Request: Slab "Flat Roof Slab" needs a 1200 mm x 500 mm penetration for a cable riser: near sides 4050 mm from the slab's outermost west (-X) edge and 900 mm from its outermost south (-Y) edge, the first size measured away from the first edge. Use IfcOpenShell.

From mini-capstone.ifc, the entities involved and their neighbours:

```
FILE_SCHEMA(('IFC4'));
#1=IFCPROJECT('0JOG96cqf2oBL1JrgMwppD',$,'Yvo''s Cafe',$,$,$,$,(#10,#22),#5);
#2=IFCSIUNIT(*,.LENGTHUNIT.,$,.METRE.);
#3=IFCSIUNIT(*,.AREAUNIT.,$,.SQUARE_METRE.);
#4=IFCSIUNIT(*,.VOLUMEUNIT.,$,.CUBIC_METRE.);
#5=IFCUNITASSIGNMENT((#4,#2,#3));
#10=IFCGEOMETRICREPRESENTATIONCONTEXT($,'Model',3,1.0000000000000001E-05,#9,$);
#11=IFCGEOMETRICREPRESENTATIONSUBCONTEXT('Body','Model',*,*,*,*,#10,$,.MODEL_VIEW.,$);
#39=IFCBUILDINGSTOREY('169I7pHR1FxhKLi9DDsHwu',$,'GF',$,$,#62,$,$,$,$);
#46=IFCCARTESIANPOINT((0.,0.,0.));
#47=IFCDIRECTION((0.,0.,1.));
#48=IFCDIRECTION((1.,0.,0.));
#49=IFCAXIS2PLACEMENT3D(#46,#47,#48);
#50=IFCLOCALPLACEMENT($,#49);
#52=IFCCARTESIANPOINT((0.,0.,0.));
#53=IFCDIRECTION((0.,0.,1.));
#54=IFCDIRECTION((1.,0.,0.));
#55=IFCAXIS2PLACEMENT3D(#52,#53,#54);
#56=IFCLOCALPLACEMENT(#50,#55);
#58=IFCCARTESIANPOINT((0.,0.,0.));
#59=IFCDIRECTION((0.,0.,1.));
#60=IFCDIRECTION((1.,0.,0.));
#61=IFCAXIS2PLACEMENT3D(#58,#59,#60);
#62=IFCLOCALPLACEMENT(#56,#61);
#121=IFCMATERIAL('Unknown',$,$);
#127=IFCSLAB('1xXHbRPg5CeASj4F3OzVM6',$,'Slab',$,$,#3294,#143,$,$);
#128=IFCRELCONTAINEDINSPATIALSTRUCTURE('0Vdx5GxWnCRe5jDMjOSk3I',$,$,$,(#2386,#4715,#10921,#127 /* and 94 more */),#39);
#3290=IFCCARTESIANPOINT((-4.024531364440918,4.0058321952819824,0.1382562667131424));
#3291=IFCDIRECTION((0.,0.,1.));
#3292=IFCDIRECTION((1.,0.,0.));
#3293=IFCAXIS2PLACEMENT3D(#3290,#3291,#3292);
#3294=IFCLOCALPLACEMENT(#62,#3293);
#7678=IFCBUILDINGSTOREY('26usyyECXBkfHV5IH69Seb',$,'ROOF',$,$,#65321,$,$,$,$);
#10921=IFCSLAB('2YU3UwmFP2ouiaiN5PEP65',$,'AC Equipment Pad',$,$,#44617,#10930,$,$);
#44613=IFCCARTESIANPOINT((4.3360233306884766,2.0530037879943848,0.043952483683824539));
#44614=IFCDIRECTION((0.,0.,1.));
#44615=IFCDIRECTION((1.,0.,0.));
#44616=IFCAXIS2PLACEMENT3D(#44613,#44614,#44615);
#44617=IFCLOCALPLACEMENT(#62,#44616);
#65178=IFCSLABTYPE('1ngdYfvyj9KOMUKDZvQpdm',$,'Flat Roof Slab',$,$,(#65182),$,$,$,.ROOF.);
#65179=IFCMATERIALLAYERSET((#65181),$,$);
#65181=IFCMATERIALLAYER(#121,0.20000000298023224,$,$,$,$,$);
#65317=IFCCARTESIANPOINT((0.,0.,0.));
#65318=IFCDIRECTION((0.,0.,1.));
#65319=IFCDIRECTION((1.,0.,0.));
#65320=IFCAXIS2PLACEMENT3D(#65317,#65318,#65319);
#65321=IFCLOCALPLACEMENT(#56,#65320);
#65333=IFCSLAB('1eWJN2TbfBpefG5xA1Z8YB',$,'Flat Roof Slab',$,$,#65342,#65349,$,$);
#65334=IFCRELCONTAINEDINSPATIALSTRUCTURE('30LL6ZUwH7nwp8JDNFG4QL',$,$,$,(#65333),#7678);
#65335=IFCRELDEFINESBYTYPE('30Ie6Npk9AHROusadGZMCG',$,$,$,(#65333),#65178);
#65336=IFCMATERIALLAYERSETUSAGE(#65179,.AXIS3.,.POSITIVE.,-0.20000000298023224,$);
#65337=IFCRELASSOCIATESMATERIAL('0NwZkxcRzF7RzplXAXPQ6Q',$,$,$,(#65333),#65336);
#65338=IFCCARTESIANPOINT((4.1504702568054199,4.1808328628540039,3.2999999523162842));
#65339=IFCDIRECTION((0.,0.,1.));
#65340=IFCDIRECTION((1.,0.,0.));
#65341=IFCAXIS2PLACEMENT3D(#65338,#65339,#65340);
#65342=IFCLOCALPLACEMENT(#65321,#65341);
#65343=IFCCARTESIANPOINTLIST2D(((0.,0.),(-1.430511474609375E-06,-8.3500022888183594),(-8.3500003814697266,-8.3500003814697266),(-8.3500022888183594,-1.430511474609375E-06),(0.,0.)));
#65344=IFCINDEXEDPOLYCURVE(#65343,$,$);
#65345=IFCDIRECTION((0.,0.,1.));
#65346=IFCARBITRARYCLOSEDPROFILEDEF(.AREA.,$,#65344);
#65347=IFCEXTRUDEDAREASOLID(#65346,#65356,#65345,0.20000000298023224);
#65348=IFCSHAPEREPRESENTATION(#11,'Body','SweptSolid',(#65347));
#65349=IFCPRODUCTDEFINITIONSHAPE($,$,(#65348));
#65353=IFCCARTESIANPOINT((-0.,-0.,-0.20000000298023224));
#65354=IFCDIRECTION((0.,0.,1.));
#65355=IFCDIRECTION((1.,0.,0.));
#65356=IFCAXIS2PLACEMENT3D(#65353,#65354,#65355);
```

```python
import numpy as np
import ifcopenshell
import ifcopenshell.api.feature
import ifcopenshell.api.geometry
import ifcopenshell.api.root
import ifcopenshell.geom
import ifcopenshell.util.placement
import ifcopenshell.util.representation
import ifcopenshell.util.shape
import ifcopenshell.util.unit

model = ifcopenshell.open("mini-capstone.ifc")
unit_scale = ifcopenshell.util.unit.calculate_unit_scale(model)
settings = ifcopenshell.geom.settings()


def volume(element):
    """Net volume in cubic metres, openings subtracted."""
    shape = ifcopenshell.geom.create_shape(settings, element)
    return ifcopenshell.util.shape.get_volume(shape.geometry)


slab = model.by_guid("1eWJN2TbfBpefG5xA1Z8YB")
before = volume(slab)

# Extent in the slab's own axes, in metres. The edges named are its -X and -Y sides.
slab_shape = ifcopenshell.geom.create_shape(settings, slab)
vertices = ifcopenshell.util.shape.get_vertices(slab_shape.geometry)
x_min, y_min, bottom = vertices.min(axis=0)
top = vertices[:, 2].max()

opening = ifcopenshell.api.root.create_entity(model, ifc_class="IfcOpeningElement", name="Cable riser opening", predefined_type="OPENING")
context = ifcopenshell.util.representation.get_context(model, "Model", "Body", "MODEL_VIEW")
width, depth = 1.2, 0.5
outline = [(0.0, 0.0), (width, 0.0), (width, depth), (0.0, depth), (0.0, 0.0)]
# Overshoot both faces by 50 mm so the cut is clean.
shape = ifcopenshell.api.geometry.add_slab_representation(
    model, context=context, depth=top - bottom + 0.1, polyline=outline
)
ifcopenshell.api.geometry.assign_representation(model, product=opening, representation=shape)

matrix = ifcopenshell.util.placement.get_local_placement(slab.ObjectPlacement)
matrix[:, 3] = matrix @ np.append(np.array([x_min + 4.05, y_min + 0.9, bottom - 0.05]) / unit_scale, 1.0)
ifcopenshell.api.geometry.edit_object_placement(model, product=opening, matrix=matrix, is_si=False)
ifcopenshell.api.feature.add_feature(model, feature=opening, element=slab)

after = volume(slab)

print(f"slab volume {before:.3f} -> {after:.3f} m3")

model.write("mini-capstone_updated.ifc")
```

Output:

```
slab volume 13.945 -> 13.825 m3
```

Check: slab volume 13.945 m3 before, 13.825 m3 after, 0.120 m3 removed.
